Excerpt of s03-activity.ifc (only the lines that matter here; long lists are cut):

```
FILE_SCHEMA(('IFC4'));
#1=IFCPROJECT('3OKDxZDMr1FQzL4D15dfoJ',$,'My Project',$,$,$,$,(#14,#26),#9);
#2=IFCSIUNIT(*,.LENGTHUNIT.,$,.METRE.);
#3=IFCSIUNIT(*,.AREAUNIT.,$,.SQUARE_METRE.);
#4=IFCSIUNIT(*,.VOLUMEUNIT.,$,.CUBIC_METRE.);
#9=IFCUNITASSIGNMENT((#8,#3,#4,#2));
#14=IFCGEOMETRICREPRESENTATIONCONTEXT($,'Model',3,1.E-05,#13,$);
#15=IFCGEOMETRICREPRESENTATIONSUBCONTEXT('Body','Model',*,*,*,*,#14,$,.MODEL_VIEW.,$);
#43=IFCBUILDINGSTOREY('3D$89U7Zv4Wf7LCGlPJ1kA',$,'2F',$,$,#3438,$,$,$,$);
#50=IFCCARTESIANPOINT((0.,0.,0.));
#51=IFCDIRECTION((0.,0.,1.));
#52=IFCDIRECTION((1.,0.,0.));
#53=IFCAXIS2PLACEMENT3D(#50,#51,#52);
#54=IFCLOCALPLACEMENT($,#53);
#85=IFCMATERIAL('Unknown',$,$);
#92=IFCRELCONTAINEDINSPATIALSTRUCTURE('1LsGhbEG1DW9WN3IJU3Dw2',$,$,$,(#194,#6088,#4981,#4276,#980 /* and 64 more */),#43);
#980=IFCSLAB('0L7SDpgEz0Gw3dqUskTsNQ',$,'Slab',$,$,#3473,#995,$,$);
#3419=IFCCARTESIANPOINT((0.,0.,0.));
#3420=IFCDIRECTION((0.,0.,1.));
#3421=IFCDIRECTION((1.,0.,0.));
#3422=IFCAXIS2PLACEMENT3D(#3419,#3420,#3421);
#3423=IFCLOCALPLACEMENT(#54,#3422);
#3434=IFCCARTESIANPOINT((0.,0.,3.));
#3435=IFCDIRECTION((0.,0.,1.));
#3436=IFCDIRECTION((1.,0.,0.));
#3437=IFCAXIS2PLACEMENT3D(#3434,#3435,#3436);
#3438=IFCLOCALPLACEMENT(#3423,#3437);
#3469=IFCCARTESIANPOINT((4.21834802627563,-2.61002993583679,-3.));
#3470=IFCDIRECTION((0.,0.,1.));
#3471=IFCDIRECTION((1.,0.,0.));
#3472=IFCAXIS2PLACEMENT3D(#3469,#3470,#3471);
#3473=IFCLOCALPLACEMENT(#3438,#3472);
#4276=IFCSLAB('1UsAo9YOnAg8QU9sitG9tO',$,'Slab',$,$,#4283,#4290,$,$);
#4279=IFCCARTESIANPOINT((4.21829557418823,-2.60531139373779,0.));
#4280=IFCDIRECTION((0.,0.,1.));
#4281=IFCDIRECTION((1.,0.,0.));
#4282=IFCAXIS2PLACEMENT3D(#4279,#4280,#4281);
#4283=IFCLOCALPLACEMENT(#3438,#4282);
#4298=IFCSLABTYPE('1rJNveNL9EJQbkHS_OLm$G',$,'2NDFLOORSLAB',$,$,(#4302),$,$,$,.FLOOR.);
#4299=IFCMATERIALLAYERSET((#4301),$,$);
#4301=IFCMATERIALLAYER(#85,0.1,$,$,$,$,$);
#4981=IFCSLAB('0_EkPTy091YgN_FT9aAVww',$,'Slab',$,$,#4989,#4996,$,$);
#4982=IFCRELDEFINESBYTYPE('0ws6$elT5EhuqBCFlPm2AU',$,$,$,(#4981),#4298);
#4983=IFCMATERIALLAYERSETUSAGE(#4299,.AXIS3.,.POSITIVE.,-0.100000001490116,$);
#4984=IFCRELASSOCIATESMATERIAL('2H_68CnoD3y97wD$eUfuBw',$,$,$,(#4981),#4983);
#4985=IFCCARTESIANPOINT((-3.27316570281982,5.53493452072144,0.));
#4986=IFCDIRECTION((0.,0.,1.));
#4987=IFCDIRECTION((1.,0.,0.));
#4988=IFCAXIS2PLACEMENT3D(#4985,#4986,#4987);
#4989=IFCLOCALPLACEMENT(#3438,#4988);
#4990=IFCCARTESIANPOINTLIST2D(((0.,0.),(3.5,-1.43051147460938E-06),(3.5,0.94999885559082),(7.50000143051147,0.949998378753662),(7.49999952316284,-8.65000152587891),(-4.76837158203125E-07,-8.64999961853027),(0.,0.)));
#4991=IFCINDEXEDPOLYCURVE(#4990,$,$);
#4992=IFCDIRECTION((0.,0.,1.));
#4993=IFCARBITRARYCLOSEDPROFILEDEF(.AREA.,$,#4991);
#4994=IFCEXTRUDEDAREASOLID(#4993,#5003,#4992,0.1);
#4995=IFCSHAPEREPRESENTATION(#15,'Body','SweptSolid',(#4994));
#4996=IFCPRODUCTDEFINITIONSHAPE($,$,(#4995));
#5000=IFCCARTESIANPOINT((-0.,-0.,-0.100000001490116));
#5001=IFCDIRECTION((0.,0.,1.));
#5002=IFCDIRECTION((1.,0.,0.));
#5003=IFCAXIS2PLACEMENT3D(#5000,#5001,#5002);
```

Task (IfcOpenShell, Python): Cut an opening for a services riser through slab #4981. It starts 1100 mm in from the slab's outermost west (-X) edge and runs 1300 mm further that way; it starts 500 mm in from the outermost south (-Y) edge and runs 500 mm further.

```python
import numpy as np
import ifcopenshell
import ifcopenshell.api.feature
import ifcopenshell.api.geometry
import ifcopenshell.api.root
import ifcopenshell.geom
import ifcopenshell.util.placement
import ifcopenshell.util.representation
import ifcopenshell.util.shape
import ifcopenshell.util.unit

model = ifcopenshell.open("s03-activity.ifc")
unit_scale = ifcopenshell.util.unit.calculate_unit_scale(model)
settings = ifcopenshell.geom.settings()


def volume(element):
    """Net volume in cubic metres, openings subtracted."""
    shape = ifcopenshell.geom.create_shape(settings, element)
    return ifcopenshell.util.shape.get_volume(shape.geometry)


slab = model.by_guid("0_EkPTy091YgN_FT9aAVww")
before = volume(slab)

# Extent in the slab's own axes, in metres. The edges named are its -X and -Y sides.
slab_shape = ifcopenshell.geom.create_shape(settings, slab)
vertices = ifcopenshell.util.shape.get_vertices(slab_shape.geometry)
x_min, y_min, bottom = vertices.min(axis=0)
top = vertices[:, 2].max()

opening = ifcopenshell.api.root.create_entity(model, ifc_class="IfcOpeningElement", name="Services riser opening", predefined_type="OPENING")
context = ifcopenshell.util.representation.get_context(model, "Model", "Body", "MODEL_VIEW")
width, depth = 1.3, 0.5
outline = [(0.0, 0.0), (width, 0.0), (width, depth), (0.0, depth), (0.0, 0.0)]
# Overshoot both faces by 50 mm so the cut is clean.
shape = ifcopenshell.api.geometry.add_slab_representation(
    model, context=context, depth=top - bottom + 0.1, polyline=outline
)
ifcopenshell.api.geometry.assign_representation(model, product=opening, representation=shape)

matrix = ifcopenshell.util.placement.get_local_placement(slab.ObjectPlacement)
matrix[:, 3] = matrix @ np.append(np.array([x_min + 1.1, y_min + 0.5, bottom - 0.05]) / unit_scale, 1.0)
ifcopenshell.api.geometry.edit_object_placement(model, product=opening, matrix=matrix, is_si=False)
ifcopenshell.api.feature.add_feature(model, feature=opening, element=slab)

after = volume(slab)

print(f"slab volume {before:.3f} -> {after:.3f} m3")

model.write("s03-activity_updated.ifc")
```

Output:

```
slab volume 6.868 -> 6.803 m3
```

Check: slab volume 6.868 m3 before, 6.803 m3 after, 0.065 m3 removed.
